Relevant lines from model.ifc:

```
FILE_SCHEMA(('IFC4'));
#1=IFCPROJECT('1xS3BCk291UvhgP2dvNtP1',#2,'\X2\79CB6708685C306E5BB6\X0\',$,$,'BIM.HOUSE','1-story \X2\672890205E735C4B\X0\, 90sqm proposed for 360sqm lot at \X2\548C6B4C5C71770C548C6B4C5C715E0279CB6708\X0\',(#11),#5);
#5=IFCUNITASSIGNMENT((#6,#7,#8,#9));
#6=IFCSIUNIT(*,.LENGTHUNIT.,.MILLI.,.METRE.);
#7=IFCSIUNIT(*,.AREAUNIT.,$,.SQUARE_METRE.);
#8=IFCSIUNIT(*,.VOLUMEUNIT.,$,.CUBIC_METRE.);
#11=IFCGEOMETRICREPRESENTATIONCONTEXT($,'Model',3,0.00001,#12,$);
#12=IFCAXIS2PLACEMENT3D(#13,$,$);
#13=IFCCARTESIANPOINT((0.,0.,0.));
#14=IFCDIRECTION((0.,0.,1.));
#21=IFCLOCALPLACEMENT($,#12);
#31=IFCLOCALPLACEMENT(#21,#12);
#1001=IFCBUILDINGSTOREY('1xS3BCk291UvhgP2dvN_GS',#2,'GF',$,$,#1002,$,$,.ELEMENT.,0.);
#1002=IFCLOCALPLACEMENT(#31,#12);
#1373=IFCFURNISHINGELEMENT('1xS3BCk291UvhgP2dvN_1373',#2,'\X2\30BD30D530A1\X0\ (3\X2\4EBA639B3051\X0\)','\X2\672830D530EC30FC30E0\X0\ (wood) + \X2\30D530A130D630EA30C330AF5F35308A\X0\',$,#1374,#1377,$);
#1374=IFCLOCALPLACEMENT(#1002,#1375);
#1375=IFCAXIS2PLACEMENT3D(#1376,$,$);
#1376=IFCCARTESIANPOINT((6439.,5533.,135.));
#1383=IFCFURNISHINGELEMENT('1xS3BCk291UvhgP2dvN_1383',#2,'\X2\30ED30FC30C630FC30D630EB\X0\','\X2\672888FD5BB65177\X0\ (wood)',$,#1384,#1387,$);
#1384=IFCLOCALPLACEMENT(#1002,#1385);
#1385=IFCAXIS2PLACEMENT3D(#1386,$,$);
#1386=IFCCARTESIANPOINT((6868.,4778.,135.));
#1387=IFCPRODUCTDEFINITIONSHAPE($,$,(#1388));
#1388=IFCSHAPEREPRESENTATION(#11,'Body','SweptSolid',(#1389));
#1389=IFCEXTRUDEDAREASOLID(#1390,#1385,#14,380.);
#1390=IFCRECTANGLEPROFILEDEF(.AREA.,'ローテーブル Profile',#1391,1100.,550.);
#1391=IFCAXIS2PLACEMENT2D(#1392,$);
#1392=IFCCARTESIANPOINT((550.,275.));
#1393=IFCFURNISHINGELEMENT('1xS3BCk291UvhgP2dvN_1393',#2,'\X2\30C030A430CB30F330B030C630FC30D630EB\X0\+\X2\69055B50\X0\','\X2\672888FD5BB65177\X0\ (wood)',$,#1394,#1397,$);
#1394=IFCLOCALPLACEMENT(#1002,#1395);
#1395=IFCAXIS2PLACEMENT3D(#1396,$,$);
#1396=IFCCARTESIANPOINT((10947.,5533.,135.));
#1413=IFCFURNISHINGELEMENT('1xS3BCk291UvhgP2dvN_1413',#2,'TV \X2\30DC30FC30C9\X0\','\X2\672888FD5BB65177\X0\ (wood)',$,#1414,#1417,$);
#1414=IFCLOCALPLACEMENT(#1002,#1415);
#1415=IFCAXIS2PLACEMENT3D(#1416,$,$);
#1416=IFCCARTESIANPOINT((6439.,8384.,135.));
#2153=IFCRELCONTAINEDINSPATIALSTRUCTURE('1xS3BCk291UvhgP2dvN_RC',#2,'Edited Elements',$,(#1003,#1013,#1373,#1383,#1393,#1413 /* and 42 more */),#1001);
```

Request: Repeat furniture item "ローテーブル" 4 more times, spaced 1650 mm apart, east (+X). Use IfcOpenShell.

```python
import numpy as np
import ifcopenshell
import ifcopenshell.api.geometry
import ifcopenshell.api.root
import ifcopenshell.util.element
import ifcopenshell.util.placement

model = ifcopenshell.open("model.ifc")


def reuse_history(source, copy):
    """copy_class also copies each property set's owner history, people and application; keep the originals."""
    for rel in copy.IsDefinedBy:
        if rel.is_a("IfcRelDefinesByProperties") and (history := rel.RelatingPropertyDefinition.OwnerHistory):
            rel.RelatingPropertyDefinition.OwnerHistory = source.OwnerHistory
            ifcopenshell.util.element.remove_deep2(model, history)


source = model.by_id(1383)
base = ifcopenshell.util.placement.get_local_placement(source.ObjectPlacement)
step = np.array([1.0, 0.0, 0.0]) * 1650.0

for i in range(1, 5):
    copy = ifcopenshell.api.root.copy_class(model, product=source)
    copy.Representation = ifcopenshell.util.element.copy_deep(
        model, source.Representation, exclude=["IfcGeometricRepresentationContext", "IfcRepresentationMap"]
    )
    reuse_history(source, copy)
    matrix = base.copy()
    matrix[:3, 3] += i * step
    print("added at", matrix[:3, 3].round(3) + 0.0)
    ifcopenshell.api.geometry.edit_object_placement(model, product=copy, matrix=matrix, is_si=False)

model.write("model_edited.ifc")
```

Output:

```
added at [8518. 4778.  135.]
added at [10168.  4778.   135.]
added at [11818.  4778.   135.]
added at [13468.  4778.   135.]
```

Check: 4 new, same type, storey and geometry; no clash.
